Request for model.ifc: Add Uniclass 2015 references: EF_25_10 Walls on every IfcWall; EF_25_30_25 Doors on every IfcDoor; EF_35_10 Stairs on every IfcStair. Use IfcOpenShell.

First a look at what the model holds.

```python
import ifcopenshell

model = ifcopenshell.open("model.ifc")
print(model.schema)
print("classifications:", [c.Name for c in model.by_type("IfcClassification")])
for ifc_class in ("IfcDoor", "IfcRoof", "IfcStair", "IfcWall", "IfcWindow"):
    print(ifc_class, len(model.by_type(ifc_class)))
```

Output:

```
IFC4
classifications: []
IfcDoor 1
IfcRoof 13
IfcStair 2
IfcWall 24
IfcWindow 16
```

```python
import ifcopenshell
import ifcopenshell.api.classification

model = ifcopenshell.open("model.ifc")

system = ifcopenshell.api.classification.add_classification(model, classification="Uniclass 2015")

codes = {
    "IfcWall": ("EF_25_10", "Walls"),
    "IfcDoor": ("EF_25_30_25", "Doors"),
    "IfcStair": ("EF_35_10", "Stairs"),
}
for ifc_class, (code, name) in codes.items():
    products = model.by_type(ifc_class)
    ifcopenshell.api.classification.add_reference(
        model, products=products, classification=system, identification=code, name=name
    )
    print(code, len(products))

model.write("model_updated.ifc")
```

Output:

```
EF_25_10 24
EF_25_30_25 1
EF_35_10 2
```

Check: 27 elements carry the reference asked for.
